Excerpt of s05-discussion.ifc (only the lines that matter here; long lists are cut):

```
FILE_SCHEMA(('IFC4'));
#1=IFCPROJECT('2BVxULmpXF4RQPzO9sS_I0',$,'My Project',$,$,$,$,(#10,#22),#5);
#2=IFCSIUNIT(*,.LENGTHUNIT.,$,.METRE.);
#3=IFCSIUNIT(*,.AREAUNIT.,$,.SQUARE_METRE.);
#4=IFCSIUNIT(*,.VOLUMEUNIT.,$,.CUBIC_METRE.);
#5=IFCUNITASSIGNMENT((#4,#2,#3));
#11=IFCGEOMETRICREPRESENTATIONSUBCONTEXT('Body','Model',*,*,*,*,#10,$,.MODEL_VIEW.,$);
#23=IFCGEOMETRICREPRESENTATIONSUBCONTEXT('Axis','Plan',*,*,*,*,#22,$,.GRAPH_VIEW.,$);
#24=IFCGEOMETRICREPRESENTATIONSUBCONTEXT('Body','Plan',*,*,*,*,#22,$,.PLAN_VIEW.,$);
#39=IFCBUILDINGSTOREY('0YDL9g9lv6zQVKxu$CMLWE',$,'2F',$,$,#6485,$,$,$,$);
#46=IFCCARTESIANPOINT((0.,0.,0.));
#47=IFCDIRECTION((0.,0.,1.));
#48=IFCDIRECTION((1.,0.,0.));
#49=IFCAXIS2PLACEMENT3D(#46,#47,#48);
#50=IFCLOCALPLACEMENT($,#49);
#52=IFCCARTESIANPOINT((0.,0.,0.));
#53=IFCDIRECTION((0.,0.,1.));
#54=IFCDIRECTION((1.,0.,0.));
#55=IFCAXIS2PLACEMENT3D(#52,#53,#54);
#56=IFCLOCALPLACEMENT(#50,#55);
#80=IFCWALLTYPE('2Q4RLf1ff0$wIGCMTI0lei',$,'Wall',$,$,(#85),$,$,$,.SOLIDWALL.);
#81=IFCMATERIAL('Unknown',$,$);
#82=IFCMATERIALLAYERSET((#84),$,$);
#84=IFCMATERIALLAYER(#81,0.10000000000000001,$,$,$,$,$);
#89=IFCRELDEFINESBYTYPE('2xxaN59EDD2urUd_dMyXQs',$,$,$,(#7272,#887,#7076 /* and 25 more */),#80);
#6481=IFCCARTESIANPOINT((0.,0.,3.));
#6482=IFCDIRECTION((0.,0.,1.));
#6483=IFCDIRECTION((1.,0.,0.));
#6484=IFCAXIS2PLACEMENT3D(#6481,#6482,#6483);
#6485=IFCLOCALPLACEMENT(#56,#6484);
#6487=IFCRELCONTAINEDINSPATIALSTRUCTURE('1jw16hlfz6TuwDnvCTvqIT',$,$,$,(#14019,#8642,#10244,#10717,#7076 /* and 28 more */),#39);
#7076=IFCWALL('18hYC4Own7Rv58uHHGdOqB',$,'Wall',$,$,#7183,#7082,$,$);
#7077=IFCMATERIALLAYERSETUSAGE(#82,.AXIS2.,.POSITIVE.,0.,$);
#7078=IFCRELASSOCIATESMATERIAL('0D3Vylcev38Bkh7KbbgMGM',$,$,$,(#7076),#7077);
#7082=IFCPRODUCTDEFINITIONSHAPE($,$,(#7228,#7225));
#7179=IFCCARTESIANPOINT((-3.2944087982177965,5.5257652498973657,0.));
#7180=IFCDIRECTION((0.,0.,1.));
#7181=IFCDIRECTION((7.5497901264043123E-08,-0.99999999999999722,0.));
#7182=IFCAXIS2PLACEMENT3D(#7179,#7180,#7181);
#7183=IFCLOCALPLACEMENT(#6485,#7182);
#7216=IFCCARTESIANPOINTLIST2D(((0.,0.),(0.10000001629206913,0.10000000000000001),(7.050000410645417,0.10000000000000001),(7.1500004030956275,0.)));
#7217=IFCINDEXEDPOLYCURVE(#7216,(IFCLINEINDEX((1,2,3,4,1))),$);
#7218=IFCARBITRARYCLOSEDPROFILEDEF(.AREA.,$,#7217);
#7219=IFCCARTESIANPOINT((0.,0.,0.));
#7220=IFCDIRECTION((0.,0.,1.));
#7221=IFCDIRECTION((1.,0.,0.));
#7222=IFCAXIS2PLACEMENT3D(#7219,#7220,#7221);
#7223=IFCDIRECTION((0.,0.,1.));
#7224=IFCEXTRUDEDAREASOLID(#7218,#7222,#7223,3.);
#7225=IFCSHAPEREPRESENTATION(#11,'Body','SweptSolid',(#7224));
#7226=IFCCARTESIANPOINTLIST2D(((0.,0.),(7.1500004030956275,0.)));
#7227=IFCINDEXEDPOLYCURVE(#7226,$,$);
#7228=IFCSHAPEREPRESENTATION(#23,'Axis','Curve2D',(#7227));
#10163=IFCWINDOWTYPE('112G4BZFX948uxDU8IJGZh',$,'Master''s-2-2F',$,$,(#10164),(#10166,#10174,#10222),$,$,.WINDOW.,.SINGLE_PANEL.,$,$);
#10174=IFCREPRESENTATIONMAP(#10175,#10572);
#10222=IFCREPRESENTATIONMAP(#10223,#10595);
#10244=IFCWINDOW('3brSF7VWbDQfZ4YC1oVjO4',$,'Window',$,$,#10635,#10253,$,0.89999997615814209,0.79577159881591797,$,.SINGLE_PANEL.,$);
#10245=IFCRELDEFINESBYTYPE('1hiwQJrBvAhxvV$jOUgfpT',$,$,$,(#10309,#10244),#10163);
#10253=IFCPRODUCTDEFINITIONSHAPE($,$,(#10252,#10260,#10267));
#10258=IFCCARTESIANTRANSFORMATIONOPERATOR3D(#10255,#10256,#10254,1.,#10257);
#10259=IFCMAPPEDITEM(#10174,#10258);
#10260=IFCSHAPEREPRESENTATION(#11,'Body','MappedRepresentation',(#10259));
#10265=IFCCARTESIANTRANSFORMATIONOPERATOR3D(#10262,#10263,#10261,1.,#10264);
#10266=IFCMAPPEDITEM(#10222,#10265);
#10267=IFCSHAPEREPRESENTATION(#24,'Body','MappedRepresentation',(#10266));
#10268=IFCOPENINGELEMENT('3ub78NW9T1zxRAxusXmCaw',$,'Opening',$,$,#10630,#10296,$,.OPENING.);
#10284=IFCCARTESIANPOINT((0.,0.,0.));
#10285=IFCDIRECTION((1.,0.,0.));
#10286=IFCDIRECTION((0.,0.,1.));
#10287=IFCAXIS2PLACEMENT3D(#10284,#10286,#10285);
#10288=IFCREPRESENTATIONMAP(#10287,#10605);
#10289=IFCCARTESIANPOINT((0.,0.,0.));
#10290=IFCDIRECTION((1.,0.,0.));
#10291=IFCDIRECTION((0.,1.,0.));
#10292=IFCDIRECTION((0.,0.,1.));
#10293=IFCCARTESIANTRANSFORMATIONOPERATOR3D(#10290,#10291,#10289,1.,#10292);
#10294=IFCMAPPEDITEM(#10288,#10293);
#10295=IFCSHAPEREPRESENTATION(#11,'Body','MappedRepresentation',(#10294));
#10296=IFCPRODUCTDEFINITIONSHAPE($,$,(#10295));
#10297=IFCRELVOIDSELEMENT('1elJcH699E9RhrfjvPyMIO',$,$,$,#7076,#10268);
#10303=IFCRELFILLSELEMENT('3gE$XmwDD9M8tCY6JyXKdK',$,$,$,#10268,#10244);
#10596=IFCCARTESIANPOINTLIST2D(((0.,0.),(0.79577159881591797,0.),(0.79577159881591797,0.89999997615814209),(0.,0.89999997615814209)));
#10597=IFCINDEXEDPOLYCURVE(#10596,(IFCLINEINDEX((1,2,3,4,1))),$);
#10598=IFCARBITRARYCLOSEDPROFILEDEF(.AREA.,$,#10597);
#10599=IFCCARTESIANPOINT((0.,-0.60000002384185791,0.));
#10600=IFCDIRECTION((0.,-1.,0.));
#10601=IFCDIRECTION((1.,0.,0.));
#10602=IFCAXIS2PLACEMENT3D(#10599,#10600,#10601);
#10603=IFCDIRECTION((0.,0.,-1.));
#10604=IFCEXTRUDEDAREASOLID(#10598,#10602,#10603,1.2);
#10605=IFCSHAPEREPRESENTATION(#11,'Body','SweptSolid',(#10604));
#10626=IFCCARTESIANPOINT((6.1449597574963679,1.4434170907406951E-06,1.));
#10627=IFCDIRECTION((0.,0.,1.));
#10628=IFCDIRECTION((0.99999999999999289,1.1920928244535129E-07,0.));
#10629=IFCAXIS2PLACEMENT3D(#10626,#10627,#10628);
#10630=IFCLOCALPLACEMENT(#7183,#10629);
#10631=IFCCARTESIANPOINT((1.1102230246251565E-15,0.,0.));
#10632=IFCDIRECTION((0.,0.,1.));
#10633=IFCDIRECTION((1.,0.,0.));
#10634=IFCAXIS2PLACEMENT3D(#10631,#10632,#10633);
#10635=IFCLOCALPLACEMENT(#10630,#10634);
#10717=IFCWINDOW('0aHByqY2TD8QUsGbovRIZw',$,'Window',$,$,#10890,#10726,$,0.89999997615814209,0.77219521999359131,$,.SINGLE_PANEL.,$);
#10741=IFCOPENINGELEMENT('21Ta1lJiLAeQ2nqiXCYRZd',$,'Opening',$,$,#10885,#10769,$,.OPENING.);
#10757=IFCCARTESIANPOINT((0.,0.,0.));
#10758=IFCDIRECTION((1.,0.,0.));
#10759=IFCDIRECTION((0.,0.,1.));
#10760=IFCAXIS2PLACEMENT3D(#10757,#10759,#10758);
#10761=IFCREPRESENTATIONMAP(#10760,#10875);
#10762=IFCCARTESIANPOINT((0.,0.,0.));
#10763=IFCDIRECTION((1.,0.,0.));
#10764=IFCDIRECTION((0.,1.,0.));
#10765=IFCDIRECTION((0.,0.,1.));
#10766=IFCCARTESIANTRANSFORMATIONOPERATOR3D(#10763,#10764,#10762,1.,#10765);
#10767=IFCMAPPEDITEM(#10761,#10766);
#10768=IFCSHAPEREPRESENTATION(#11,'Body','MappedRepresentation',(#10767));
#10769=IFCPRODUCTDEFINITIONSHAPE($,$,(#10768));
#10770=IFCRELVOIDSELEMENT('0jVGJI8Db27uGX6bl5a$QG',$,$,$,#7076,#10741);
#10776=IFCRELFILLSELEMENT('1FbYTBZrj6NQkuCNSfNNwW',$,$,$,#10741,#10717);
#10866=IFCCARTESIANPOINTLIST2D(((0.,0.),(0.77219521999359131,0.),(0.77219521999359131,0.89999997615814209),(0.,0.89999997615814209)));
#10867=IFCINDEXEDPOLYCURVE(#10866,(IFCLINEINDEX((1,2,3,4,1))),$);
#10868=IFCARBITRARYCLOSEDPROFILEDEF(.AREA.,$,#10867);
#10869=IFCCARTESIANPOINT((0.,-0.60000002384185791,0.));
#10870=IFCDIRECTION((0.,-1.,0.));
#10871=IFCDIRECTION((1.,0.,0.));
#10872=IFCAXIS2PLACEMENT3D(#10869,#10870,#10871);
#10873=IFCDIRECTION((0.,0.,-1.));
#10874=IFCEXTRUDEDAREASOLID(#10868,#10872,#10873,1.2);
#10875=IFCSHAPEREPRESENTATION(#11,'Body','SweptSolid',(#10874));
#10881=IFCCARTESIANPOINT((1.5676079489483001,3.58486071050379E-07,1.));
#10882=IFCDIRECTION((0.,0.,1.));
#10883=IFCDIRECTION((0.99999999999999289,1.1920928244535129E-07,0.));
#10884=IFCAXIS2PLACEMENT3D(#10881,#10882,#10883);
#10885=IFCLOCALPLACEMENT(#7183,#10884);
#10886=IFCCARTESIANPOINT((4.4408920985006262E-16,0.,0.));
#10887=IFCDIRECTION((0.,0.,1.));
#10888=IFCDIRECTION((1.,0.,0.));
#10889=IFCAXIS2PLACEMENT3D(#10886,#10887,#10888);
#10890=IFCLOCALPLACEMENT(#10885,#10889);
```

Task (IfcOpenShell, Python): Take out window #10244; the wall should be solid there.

```python
import ifcopenshell
import ifcopenshell.api.feature
import ifcopenshell.api.root
import ifcopenshell.geom
import ifcopenshell.util.shape

model = ifcopenshell.open("s05-discussion.ifc")
settings = ifcopenshell.geom.settings()


def volume(element):
    """Net volume in cubic metres, openings subtracted."""
    shape = ifcopenshell.geom.create_shape(settings, element)
    return ifcopenshell.util.shape.get_volume(shape.geometry)


window = model.by_id(10244)
opening = window.FillsVoids[0].RelatingOpeningElement
wall = opening.VoidsElements[0].RelatingBuildingElement
before = volume(wall)

ifcopenshell.api.root.remove_product(model, product=window)
ifcopenshell.api.feature.remove_feature(model, feature=opening)

after = volume(wall)

print(f"wall volume {before:.3f} -> {after:.3f} m3")

model.write("s05-discussion_v2.ifc")
```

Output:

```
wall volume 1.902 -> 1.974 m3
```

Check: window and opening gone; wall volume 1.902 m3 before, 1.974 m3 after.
